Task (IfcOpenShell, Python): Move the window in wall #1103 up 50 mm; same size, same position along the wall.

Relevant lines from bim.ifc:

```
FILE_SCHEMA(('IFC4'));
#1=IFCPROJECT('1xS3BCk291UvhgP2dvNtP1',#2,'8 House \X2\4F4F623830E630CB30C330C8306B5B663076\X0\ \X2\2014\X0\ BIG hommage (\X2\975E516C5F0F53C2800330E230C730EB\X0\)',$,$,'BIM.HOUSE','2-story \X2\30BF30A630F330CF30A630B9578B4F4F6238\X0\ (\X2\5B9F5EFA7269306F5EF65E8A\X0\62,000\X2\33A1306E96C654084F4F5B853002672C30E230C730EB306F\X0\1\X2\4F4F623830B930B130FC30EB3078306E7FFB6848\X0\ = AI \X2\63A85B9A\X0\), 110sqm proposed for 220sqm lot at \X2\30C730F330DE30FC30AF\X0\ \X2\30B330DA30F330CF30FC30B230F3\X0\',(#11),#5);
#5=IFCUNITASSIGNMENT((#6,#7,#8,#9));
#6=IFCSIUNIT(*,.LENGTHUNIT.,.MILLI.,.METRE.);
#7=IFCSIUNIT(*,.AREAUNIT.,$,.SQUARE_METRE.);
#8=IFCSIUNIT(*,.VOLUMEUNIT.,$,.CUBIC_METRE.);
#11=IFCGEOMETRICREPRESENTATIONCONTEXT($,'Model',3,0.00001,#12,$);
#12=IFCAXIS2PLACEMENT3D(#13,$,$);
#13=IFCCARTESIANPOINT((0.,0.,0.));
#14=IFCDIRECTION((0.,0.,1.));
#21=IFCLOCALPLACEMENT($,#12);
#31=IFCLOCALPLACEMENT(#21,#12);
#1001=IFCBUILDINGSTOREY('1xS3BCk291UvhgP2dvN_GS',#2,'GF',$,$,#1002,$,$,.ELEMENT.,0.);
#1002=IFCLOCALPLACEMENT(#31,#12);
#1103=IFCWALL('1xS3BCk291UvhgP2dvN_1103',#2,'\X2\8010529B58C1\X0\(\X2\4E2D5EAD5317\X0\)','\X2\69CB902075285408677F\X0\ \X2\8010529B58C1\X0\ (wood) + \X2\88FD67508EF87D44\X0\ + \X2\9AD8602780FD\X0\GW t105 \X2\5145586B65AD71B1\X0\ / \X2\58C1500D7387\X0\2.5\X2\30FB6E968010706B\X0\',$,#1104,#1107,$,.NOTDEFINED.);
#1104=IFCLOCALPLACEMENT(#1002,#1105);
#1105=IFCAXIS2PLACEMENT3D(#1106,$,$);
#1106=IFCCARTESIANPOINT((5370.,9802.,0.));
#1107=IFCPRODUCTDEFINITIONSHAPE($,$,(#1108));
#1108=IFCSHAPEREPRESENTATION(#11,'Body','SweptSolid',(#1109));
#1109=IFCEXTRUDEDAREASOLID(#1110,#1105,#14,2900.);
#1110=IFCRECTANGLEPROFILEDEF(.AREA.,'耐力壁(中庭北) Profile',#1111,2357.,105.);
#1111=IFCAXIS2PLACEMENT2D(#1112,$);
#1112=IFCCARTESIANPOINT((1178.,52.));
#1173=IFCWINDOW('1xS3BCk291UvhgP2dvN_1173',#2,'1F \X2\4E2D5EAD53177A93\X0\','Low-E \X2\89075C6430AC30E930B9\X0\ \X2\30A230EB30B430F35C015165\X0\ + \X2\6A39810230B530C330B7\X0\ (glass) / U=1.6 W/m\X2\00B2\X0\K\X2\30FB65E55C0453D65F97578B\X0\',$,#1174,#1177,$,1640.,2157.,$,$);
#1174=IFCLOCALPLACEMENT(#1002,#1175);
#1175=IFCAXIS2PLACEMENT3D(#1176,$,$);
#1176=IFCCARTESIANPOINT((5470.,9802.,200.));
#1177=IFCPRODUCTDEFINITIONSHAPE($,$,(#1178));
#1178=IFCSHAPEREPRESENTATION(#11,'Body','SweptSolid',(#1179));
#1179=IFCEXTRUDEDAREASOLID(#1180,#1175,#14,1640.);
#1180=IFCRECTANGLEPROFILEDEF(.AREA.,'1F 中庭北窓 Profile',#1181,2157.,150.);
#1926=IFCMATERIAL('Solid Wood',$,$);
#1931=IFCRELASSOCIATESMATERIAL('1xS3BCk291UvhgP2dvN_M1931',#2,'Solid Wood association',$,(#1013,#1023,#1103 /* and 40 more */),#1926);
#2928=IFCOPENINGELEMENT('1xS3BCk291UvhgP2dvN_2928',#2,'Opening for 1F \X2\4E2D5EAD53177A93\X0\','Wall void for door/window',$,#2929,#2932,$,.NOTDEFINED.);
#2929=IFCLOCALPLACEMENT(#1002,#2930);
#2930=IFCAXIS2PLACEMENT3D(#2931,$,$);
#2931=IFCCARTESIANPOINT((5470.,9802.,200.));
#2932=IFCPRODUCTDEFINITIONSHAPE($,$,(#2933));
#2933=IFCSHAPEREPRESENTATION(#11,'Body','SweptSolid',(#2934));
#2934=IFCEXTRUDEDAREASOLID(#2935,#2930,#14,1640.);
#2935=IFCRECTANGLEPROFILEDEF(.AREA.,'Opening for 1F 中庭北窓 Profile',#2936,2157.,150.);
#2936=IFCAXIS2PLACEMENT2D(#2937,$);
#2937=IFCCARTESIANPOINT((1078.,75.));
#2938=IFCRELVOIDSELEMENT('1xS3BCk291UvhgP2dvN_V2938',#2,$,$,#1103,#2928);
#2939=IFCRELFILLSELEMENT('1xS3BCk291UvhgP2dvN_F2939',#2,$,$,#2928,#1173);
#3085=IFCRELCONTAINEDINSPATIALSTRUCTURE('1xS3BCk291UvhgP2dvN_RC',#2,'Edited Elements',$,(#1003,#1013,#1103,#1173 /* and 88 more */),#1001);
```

```python
import numpy as np
import ifcopenshell
import ifcopenshell.api.geometry
import ifcopenshell.util.placement
import ifcopenshell.util.unit

model = ifcopenshell.open("bim.ifc")
unit_scale = ifcopenshell.util.unit.calculate_unit_scale(model)

window = model.by_guid("1xS3BCk291UvhgP2dvN_1173")
opening = window.FillsVoids[0].RelatingOpeningElement
dz = 0.05 / unit_scale

shift = np.array([0.0, 0.0, dz])
# The window is not placed relative to its opening, so move both.
for product in (opening, window):
    matrix = ifcopenshell.util.placement.get_local_placement(product.ObjectPlacement)
    matrix[:3, 3] += shift
    ifcopenshell.api.geometry.edit_object_placement(model, product=product, matrix=matrix, is_si=False)

print(f"moved by {dz * unit_scale:+.3f} m")

model.write("bim_rev.ifc")
```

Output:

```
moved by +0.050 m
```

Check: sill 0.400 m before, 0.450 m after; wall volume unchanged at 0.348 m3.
